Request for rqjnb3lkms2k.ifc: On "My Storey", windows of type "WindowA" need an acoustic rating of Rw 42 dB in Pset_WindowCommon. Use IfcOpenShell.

First a look at what the model holds.

```python
import ifcopenshell
import ifcopenshell.util.element

model = ifcopenshell.open("rqjnb3lkms2k.ifc")
print(model.schema)
storey = next(s for s in model.by_type("IfcBuildingStorey") if s.Name == "My Storey")
windows = [e for e in ifcopenshell.util.element.get_decomposition(storey) if e.is_a("IfcWindow")]
seen = {}
for e in windows:
    element_type = ifcopenshell.util.element.get_type(e)
    key = (element_type.Name if element_type != e and element_type else None, ifcopenshell.util.element.get_pset(e, "Pset_WindowCommon", "AcousticRating"))
    seen[key] = seen.get(key, 0) + 1
for (name, value), count in sorted(seen.items(), key=str):
    print(count, "x", name, "|", value)
```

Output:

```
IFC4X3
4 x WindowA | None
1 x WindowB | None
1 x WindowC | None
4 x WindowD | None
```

```python
import ifcopenshell
import ifcopenshell.api.pset
import ifcopenshell.util.element

model = ifcopenshell.open("rqjnb3lkms2k.ifc")

storey = next(s for s in model.by_type("IfcBuildingStorey") if s.Name == "My Storey")
windows = [e for e in ifcopenshell.util.element.get_decomposition(storey) if e.is_a("IfcWindow")]

count = 0
for e in windows:
    element_type = ifcopenshell.util.element.get_type(e)
    if element_type in (None, e) or element_type.Name != "WindowA":
        continue
    # add_pset returns the element's existing set when there is one.
    pset = ifcopenshell.api.pset.add_pset(model, product=e, name="Pset_WindowCommon")
    ifcopenshell.api.pset.edit_pset(model, pset=pset, properties={"AcousticRating": "Rw 42 dB"})
    count += 1

print(count, "windows updated")

model.write("rqjnb3lkms2k_v2.ifc")
```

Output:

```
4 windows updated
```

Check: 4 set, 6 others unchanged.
